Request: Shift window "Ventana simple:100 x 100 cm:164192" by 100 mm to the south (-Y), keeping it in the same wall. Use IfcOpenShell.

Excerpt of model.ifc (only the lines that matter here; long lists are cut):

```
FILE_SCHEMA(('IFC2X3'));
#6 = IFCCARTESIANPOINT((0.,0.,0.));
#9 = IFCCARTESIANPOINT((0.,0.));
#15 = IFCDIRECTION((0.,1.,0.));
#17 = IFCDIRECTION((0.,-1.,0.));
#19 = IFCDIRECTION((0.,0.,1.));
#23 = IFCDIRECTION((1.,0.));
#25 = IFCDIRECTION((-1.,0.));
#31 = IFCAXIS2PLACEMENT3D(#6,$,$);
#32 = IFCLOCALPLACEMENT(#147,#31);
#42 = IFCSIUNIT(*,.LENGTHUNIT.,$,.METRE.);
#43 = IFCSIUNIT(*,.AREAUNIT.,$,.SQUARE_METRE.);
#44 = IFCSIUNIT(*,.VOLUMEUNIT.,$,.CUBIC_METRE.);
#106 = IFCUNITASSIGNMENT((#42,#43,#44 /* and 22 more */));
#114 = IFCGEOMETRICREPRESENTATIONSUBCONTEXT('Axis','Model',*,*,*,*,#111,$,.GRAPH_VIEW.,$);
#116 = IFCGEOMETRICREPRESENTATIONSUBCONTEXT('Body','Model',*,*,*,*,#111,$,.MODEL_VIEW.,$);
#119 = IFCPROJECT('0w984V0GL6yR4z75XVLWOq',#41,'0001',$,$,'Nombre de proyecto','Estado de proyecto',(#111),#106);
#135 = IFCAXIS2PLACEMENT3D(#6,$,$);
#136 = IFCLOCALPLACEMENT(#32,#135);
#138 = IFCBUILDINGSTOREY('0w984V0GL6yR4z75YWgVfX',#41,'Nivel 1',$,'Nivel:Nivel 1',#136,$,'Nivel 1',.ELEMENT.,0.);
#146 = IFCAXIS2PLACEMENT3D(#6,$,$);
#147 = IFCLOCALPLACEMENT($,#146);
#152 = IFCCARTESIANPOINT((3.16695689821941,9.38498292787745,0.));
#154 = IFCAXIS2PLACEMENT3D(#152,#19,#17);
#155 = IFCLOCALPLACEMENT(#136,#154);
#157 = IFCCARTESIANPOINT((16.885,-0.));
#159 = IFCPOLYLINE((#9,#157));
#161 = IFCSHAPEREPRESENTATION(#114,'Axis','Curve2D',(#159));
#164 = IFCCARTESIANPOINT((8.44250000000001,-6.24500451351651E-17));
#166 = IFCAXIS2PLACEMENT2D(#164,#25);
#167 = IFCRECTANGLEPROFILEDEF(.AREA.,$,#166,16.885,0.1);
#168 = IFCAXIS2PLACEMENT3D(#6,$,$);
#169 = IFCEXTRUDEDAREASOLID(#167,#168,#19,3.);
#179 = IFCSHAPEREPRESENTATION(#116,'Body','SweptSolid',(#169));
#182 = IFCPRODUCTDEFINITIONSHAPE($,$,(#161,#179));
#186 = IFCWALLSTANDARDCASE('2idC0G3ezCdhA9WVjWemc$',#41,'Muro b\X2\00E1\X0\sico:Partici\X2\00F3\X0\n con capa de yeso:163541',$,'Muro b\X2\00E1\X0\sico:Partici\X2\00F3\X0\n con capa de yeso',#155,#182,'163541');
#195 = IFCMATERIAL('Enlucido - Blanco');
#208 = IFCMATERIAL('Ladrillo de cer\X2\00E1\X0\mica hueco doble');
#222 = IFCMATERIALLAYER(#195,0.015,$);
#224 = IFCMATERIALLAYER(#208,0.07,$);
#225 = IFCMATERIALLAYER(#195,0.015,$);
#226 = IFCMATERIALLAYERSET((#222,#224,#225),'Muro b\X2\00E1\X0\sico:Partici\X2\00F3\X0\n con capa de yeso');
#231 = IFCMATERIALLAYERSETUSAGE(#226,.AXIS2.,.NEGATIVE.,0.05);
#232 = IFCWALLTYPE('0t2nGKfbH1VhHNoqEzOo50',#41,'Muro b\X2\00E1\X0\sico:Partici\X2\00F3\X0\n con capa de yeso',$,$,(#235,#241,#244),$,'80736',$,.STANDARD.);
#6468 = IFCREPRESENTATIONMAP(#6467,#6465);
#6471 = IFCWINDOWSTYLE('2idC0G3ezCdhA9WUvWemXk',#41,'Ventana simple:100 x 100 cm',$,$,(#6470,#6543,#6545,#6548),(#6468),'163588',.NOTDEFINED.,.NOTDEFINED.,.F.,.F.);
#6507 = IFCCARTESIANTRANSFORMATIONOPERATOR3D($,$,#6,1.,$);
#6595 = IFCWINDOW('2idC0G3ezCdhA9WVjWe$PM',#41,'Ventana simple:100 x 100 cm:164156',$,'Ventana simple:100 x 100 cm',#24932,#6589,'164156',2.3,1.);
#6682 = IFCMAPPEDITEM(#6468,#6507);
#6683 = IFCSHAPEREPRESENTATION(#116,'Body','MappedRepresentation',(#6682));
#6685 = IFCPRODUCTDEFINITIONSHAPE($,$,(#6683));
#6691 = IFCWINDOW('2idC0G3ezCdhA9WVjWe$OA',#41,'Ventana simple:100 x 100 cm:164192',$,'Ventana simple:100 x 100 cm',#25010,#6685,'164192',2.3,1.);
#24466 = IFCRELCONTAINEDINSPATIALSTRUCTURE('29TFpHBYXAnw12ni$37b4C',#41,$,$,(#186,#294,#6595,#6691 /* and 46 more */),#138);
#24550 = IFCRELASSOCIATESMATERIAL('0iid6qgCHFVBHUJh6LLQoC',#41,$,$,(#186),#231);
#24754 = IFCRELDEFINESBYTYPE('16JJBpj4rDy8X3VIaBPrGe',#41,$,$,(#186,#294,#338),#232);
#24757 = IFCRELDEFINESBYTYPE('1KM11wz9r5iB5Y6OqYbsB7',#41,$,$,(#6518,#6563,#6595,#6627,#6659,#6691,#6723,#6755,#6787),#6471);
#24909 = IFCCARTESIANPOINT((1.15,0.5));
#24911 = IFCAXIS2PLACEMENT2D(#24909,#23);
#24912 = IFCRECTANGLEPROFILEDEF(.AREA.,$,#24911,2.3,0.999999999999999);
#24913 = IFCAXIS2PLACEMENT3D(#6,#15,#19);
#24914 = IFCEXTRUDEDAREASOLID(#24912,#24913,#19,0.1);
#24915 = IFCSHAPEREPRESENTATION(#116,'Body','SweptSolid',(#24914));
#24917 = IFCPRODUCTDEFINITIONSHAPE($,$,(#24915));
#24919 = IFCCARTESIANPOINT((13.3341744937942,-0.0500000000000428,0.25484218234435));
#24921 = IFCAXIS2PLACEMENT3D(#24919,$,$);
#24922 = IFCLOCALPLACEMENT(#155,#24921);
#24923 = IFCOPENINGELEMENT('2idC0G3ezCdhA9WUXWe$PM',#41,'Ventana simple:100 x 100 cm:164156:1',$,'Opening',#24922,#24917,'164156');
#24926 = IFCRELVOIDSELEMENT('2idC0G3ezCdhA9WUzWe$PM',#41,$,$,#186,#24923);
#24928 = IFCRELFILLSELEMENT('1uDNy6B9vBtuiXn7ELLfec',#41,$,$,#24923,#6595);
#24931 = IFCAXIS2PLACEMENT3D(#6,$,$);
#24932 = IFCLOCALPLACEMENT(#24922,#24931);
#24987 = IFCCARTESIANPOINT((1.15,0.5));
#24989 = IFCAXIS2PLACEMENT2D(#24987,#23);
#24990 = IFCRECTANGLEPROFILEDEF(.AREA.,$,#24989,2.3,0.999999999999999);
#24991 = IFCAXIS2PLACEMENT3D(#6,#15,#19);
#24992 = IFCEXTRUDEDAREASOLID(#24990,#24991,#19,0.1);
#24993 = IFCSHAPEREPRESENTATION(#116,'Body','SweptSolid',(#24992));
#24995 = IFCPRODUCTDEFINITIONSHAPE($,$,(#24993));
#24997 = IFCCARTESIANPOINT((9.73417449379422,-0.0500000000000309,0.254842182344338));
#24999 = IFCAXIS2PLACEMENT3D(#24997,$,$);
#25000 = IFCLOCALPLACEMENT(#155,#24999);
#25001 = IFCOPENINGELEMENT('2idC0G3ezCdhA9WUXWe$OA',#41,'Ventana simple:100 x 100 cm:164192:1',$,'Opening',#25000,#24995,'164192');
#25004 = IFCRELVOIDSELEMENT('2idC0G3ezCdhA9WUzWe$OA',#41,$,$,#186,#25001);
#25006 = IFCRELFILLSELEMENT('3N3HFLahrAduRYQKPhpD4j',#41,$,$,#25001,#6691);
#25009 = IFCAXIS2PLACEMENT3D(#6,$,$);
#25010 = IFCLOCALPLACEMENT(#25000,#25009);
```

```python
import ifcopenshell
import ifcopenshell.api.geometry
import ifcopenshell.util.placement
import ifcopenshell.util.unit

model = ifcopenshell.open("model.ifc")
unit_scale = ifcopenshell.util.unit.calculate_unit_scale(model)

window = model.by_guid("2idC0G3ezCdhA9WVjWe$OA")
opening = window.FillsVoids[0].RelatingOpeningElement
wall = opening.VoidsElements[0].RelatingBuildingElement

wall_matrix = ifcopenshell.util.placement.get_local_placement(wall.ObjectPlacement)
shift = wall_matrix[:3, 0] * 0.1 / unit_scale
before = ifcopenshell.util.placement.get_local_placement(window.ObjectPlacement)[:3, 3].copy()

# The window is placed relative to its opening, so it follows when the opening moves.
matrix = ifcopenshell.util.placement.get_local_placement(opening.ObjectPlacement)
matrix[:3, 3] += shift
ifcopenshell.api.geometry.edit_object_placement(
    model, product=opening, matrix=matrix, is_si=False, should_transform_children=True
)

after = ifcopenshell.util.placement.get_local_placement(window.ObjectPlacement)[:3, 3]
print("window moved by", (after - before).round(3) + 0.0)

model.write("model_updated.ifc")
```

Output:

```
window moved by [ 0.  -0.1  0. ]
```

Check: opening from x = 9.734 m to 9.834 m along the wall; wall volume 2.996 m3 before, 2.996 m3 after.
